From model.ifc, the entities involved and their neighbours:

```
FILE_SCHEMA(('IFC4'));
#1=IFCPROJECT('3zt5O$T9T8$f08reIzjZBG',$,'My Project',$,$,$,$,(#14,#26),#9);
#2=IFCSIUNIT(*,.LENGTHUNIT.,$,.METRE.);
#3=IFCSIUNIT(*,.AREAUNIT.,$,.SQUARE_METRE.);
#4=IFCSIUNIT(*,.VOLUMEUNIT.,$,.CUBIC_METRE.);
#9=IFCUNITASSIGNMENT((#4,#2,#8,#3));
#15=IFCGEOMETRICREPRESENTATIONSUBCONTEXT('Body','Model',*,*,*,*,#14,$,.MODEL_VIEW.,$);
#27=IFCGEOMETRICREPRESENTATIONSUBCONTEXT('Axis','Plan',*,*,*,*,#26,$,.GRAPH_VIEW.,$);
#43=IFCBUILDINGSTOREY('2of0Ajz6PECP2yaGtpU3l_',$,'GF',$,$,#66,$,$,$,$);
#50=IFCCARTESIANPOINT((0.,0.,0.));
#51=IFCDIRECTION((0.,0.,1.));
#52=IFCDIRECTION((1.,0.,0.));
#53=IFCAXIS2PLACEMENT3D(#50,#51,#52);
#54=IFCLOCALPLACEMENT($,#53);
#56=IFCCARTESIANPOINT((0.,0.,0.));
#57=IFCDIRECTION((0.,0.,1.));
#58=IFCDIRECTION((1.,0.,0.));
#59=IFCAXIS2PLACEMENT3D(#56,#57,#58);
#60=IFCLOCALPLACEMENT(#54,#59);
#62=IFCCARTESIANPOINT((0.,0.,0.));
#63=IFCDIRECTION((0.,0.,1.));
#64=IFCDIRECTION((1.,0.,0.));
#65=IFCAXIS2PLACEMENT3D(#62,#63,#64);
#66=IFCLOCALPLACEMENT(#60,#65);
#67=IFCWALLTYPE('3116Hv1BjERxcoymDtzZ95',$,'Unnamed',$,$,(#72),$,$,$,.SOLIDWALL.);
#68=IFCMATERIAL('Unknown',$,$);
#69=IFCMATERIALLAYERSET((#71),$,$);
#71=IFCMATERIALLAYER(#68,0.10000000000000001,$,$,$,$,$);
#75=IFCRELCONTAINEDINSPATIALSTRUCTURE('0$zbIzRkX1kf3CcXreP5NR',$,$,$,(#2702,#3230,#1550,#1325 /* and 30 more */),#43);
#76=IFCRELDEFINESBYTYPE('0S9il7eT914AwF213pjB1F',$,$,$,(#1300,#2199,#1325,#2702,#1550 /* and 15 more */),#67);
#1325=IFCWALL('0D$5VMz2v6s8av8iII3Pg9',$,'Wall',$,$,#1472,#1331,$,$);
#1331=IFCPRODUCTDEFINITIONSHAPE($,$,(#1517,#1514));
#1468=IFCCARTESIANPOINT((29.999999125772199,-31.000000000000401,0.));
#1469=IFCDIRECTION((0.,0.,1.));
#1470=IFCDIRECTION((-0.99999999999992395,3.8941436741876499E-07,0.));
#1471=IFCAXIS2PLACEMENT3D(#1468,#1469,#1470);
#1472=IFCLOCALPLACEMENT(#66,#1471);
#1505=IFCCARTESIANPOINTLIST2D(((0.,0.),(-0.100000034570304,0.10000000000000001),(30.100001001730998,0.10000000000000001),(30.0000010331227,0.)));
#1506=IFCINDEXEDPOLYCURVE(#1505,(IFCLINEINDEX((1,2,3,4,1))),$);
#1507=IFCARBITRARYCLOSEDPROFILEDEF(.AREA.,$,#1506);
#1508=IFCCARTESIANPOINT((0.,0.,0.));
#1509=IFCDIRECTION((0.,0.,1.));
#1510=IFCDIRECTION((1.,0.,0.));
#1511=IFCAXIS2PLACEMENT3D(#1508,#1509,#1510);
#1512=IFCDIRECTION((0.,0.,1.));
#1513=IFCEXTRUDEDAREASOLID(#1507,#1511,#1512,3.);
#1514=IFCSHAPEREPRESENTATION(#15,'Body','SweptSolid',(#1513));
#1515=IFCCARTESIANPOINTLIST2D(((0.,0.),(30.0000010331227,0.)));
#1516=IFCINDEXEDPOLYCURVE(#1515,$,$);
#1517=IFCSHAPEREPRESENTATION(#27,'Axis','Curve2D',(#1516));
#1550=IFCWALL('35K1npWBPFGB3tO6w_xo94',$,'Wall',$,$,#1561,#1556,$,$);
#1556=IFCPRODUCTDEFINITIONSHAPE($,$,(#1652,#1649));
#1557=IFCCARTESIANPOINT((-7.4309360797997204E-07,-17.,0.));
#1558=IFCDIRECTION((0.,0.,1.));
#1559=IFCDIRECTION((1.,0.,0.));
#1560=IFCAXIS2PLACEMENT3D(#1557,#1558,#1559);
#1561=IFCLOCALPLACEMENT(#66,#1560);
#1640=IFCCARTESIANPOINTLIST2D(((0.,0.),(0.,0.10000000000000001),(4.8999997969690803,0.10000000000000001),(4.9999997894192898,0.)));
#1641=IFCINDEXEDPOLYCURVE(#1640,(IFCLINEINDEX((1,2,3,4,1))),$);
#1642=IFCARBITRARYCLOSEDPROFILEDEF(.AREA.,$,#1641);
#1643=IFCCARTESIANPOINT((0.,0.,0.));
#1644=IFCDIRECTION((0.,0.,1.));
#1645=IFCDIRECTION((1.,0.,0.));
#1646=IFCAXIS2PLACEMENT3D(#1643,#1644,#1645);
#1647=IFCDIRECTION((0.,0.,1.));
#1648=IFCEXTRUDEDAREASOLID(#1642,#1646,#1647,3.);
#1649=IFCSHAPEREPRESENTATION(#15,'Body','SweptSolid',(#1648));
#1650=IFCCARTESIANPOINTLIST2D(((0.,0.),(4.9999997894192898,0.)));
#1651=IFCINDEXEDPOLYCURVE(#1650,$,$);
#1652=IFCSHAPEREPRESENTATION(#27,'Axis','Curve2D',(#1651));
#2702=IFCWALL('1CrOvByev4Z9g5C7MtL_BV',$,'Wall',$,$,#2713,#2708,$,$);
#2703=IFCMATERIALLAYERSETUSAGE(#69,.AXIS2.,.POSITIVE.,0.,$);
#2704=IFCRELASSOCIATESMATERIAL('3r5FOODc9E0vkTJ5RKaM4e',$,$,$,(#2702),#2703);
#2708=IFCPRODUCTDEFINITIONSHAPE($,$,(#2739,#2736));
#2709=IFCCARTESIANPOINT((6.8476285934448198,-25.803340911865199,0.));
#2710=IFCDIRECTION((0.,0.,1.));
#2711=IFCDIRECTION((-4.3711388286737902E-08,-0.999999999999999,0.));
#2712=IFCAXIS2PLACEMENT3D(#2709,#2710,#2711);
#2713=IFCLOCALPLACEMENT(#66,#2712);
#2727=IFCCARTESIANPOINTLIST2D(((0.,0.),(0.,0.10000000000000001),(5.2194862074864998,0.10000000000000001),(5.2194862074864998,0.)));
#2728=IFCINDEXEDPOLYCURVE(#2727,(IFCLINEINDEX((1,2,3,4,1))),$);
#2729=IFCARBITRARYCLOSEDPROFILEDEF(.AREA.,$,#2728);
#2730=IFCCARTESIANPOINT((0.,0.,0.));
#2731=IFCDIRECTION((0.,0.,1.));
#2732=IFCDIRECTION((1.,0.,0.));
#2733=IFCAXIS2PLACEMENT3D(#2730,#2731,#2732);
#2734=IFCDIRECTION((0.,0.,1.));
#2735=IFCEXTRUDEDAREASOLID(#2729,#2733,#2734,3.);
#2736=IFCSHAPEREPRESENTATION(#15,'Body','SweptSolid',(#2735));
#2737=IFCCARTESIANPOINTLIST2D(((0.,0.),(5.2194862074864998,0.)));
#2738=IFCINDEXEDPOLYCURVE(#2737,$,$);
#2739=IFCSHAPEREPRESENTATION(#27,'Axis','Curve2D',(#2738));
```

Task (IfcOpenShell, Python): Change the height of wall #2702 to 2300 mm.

```python
import ifcopenshell
import ifcopenshell.geom
import ifcopenshell.util.representation
import ifcopenshell.util.shape

model = ifcopenshell.open("model.ifc")
settings = ifcopenshell.geom.settings()


def volume(element):
    """Net volume in cubic metres, openings subtracted."""
    shape = ifcopenshell.geom.create_shape(settings, element)
    return ifcopenshell.util.shape.get_volume(shape.geometry)


wall = model.by_id(2702)
before = volume(wall)

body = ifcopenshell.util.representation.get_representation(wall, "Model", "Body")
solid = body.Items[0]
old_height = solid.Depth
solid.Depth = 2.3
after = volume(wall)

print(f"height {old_height:g} -> {solid.Depth:g}, volume {before:.3f} -> {after:.3f} m3")

model.write("model-out.ifc")
```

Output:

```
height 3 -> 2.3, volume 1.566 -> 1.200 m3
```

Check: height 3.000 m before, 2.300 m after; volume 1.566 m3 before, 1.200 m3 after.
